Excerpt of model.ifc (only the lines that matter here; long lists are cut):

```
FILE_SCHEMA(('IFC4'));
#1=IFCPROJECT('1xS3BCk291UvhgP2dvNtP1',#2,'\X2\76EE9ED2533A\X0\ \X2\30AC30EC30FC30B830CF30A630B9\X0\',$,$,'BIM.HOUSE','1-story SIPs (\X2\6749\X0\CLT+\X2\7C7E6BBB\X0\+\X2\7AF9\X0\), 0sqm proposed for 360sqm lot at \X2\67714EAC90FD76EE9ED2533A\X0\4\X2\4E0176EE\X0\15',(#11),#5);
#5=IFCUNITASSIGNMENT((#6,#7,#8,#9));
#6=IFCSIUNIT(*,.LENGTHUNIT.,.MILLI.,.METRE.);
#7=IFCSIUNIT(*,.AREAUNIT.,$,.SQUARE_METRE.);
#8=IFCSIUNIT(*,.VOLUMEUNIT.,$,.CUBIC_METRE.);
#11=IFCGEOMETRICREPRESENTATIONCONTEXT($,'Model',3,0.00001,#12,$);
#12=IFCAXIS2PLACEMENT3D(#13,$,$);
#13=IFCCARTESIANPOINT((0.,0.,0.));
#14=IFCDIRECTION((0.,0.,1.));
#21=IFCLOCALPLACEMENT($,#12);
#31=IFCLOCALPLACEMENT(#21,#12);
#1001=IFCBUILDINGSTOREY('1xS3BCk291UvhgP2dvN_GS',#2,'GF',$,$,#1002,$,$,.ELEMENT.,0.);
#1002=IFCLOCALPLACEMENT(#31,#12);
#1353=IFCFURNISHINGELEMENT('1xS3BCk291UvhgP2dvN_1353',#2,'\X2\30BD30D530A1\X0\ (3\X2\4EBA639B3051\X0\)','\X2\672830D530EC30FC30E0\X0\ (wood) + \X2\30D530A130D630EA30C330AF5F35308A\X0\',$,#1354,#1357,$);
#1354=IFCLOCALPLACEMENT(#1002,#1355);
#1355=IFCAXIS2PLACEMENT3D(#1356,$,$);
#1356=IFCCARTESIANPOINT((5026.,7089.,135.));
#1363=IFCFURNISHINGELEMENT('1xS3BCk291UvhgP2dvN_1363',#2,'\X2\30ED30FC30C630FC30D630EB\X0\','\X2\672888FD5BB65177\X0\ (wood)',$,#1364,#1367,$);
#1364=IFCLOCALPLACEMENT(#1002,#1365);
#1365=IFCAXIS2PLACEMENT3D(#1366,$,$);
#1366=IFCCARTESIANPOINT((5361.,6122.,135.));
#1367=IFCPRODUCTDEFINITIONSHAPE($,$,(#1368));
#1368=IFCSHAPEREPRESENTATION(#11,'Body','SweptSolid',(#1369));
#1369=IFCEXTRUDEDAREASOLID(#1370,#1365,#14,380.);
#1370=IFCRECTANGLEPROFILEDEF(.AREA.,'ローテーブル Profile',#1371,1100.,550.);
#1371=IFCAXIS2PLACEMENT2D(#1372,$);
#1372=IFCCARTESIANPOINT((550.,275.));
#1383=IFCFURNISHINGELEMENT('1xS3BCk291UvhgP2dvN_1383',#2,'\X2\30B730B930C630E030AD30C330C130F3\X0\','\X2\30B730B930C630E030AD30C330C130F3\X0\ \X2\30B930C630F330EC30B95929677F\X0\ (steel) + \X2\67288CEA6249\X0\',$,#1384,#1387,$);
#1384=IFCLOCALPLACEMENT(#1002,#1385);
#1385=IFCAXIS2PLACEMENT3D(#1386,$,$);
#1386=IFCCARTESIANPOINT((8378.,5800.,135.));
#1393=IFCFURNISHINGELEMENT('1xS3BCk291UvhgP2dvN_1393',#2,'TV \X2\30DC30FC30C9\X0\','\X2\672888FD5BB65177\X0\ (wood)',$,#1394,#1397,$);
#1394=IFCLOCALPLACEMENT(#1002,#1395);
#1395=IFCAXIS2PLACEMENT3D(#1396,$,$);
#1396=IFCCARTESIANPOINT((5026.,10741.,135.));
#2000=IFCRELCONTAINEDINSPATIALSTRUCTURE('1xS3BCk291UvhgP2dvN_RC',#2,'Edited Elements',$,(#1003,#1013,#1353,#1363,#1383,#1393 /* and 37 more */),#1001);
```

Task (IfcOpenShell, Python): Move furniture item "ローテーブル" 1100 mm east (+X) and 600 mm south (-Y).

```python
import ifcopenshell
import ifcopenshell.api.geometry
import ifcopenshell.util.placement
import ifcopenshell.util.unit

model = ifcopenshell.open("model.ifc")
unit_scale = ifcopenshell.util.unit.calculate_unit_scale(model)

item = model.by_id(1363)
matrix = ifcopenshell.util.placement.get_local_placement(item.ObjectPlacement)
matrix[0, 3] += 1.1 / unit_scale
matrix[1, 3] -= 0.6 / unit_scale
ifcopenshell.api.geometry.edit_object_placement(model, product=item, matrix=matrix, is_si=False)

print(ifcopenshell.util.placement.get_local_placement(item.ObjectPlacement).round(3) + 0.0)

model.write("model_v2.ifc")
```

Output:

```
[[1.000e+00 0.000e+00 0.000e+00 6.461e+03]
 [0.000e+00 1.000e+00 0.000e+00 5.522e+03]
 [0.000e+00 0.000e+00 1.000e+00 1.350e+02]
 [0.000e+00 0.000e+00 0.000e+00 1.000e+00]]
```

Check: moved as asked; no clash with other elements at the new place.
